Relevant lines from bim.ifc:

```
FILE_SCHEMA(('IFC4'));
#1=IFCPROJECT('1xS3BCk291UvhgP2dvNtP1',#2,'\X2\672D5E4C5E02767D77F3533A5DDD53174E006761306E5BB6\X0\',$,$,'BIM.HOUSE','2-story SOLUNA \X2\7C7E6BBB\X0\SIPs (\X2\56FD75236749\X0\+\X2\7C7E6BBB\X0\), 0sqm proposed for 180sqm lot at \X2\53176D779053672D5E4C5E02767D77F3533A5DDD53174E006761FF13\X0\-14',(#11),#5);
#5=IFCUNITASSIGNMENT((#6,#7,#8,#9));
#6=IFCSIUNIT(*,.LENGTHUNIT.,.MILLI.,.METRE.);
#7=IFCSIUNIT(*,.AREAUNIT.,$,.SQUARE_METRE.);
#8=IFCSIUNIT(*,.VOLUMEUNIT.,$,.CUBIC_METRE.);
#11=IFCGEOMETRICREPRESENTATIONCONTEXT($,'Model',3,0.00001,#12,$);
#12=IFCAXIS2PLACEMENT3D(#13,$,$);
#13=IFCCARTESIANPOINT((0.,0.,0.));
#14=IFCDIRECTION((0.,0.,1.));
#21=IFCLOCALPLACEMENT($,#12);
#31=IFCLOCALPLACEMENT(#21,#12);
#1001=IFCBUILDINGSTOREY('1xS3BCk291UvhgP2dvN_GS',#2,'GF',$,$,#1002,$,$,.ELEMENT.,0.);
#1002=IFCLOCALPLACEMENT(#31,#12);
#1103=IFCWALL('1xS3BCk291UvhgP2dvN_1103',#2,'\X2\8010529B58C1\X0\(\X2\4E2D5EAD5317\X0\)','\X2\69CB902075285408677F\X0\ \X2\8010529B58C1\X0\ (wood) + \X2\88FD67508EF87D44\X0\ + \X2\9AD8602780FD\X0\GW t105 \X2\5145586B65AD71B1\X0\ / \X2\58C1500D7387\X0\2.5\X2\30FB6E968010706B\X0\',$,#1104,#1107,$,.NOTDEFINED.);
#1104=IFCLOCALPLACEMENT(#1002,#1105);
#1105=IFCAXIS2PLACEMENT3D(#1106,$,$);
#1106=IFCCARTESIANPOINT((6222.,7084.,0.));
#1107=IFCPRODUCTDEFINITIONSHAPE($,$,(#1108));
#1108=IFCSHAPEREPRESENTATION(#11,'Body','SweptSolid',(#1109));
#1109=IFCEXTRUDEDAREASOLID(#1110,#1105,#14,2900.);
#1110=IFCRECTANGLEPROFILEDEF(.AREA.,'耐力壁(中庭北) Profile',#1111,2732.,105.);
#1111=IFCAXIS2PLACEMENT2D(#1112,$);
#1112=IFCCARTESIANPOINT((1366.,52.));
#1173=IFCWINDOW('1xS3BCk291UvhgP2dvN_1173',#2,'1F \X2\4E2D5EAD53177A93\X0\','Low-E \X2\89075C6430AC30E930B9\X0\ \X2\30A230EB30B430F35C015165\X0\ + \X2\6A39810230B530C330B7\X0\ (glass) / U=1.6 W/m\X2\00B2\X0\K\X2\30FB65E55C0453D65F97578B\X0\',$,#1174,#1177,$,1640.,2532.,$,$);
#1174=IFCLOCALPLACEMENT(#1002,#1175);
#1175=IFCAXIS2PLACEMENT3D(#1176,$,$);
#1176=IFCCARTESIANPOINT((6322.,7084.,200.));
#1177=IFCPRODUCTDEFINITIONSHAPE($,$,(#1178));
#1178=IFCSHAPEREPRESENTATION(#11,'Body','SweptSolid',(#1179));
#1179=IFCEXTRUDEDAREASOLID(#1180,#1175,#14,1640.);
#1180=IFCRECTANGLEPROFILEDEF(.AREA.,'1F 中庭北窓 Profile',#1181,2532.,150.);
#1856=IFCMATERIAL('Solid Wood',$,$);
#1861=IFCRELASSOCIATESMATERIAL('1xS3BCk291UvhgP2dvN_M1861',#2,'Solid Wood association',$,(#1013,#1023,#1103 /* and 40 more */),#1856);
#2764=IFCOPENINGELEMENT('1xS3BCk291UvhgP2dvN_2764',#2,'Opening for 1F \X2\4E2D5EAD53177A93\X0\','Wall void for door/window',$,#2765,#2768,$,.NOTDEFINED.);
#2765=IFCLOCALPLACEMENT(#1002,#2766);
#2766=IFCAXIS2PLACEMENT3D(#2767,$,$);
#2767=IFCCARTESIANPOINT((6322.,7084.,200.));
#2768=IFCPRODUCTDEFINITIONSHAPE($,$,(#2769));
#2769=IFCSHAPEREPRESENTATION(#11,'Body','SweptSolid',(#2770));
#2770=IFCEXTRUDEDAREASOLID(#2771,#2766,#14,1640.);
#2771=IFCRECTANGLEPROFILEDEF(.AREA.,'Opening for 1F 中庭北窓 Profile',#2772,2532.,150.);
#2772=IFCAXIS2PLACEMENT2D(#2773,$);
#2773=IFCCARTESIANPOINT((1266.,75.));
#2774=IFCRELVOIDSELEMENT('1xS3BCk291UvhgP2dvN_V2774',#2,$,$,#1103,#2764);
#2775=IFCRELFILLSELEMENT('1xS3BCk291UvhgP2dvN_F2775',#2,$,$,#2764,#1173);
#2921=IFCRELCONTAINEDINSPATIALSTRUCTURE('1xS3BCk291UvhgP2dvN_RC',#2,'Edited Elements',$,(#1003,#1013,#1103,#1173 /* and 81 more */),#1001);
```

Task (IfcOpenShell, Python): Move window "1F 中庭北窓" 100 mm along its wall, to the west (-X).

```python
import ifcopenshell
import ifcopenshell.api.geometry
import ifcopenshell.util.placement
import ifcopenshell.util.unit

model = ifcopenshell.open("bim.ifc")
unit_scale = ifcopenshell.util.unit.calculate_unit_scale(model)

window = model.by_id(1173)
opening = window.FillsVoids[0].RelatingOpeningElement
wall = opening.VoidsElements[0].RelatingBuildingElement

wall_matrix = ifcopenshell.util.placement.get_local_placement(wall.ObjectPlacement)
shift = wall_matrix[:3, 0] * -0.1 / unit_scale
before = ifcopenshell.util.placement.get_local_placement(window.ObjectPlacement)[:3, 3].copy()

# The window is not placed relative to its opening, so move both.
for product in (opening, window):
    matrix = ifcopenshell.util.placement.get_local_placement(product.ObjectPlacement)
    matrix[:3, 3] += shift
    ifcopenshell.api.geometry.edit_object_placement(model, product=product, matrix=matrix, is_si=False)

after = ifcopenshell.util.placement.get_local_placement(window.ObjectPlacement)[:3, 3]
print("window moved by", (after - before).round(3) + 0.0)

model.write("bim_rev.ifc")
```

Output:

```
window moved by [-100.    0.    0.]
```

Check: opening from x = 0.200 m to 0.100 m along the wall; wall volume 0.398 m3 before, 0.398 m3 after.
